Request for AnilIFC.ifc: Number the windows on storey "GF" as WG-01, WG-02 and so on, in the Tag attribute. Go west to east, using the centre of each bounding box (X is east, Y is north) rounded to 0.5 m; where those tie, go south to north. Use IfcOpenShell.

First a look at what the model holds.

```python
import ifcopenshell
import ifcopenshell.util.element
import ifcopenshell.util.placement

model = ifcopenshell.open("AnilIFC.ifc")
print(model.schema)
storey = next(s for s in model.by_type("IfcBuildingStorey") if s.Name == "GF")
windows = [e for e in ifcopenshell.util.element.get_decomposition(storey) if e.is_a("IfcWindow")]
for e in sorted(windows, key=lambda e: e.id()):
    origin = ifcopenshell.util.placement.get_local_placement(e.ObjectPlacement)[:3, 3]
    print(e.id(), e.Tag, e.Name, origin.round(2) + 0.0, sep=" | ")
```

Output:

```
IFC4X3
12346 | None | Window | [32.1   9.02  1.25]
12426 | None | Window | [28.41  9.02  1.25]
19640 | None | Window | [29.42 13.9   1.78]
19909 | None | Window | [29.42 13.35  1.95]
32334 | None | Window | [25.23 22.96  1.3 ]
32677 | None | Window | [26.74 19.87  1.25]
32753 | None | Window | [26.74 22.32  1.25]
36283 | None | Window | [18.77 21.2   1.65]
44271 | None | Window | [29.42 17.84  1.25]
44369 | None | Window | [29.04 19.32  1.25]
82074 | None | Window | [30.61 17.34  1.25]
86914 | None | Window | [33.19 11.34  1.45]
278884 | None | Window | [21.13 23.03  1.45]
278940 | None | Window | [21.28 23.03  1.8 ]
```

```python
import ifcopenshell
import ifcopenshell.geom
import ifcopenshell.util.element
import ifcopenshell.util.shape

model = ifcopenshell.open("AnilIFC.ifc")
settings = ifcopenshell.geom.settings()
settings.set("use-world-coords", True)


def centre(element):
    shape = ifcopenshell.geom.create_shape(settings, element)
    return ifcopenshell.util.shape.get_bbox_centroid(shape.geometry)


storey = next(s for s in model.by_type("IfcBuildingStorey") if s.Name == "GF")
windows = [e for e in ifcopenshell.util.element.get_decomposition(storey) if e.is_a("IfcWindow")]

# Insertion points can sit at a corner or the storey origin, so sort by the geometry (in metres).
centres = {e: centre(e) for e in windows}
windows.sort(key=lambda e: (round(centres[e][0] / 0.5), centres[e][1]))

for i, e in enumerate(windows, start=1):
    number = f"WG-{i:02d}"
    e.Tag = number
    print(e.id(), number)

model.write("AnilIFC-out.ifc")
```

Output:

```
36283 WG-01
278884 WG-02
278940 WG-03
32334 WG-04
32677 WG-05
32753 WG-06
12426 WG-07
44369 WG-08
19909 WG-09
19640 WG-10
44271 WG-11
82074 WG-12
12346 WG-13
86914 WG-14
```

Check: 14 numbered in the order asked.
